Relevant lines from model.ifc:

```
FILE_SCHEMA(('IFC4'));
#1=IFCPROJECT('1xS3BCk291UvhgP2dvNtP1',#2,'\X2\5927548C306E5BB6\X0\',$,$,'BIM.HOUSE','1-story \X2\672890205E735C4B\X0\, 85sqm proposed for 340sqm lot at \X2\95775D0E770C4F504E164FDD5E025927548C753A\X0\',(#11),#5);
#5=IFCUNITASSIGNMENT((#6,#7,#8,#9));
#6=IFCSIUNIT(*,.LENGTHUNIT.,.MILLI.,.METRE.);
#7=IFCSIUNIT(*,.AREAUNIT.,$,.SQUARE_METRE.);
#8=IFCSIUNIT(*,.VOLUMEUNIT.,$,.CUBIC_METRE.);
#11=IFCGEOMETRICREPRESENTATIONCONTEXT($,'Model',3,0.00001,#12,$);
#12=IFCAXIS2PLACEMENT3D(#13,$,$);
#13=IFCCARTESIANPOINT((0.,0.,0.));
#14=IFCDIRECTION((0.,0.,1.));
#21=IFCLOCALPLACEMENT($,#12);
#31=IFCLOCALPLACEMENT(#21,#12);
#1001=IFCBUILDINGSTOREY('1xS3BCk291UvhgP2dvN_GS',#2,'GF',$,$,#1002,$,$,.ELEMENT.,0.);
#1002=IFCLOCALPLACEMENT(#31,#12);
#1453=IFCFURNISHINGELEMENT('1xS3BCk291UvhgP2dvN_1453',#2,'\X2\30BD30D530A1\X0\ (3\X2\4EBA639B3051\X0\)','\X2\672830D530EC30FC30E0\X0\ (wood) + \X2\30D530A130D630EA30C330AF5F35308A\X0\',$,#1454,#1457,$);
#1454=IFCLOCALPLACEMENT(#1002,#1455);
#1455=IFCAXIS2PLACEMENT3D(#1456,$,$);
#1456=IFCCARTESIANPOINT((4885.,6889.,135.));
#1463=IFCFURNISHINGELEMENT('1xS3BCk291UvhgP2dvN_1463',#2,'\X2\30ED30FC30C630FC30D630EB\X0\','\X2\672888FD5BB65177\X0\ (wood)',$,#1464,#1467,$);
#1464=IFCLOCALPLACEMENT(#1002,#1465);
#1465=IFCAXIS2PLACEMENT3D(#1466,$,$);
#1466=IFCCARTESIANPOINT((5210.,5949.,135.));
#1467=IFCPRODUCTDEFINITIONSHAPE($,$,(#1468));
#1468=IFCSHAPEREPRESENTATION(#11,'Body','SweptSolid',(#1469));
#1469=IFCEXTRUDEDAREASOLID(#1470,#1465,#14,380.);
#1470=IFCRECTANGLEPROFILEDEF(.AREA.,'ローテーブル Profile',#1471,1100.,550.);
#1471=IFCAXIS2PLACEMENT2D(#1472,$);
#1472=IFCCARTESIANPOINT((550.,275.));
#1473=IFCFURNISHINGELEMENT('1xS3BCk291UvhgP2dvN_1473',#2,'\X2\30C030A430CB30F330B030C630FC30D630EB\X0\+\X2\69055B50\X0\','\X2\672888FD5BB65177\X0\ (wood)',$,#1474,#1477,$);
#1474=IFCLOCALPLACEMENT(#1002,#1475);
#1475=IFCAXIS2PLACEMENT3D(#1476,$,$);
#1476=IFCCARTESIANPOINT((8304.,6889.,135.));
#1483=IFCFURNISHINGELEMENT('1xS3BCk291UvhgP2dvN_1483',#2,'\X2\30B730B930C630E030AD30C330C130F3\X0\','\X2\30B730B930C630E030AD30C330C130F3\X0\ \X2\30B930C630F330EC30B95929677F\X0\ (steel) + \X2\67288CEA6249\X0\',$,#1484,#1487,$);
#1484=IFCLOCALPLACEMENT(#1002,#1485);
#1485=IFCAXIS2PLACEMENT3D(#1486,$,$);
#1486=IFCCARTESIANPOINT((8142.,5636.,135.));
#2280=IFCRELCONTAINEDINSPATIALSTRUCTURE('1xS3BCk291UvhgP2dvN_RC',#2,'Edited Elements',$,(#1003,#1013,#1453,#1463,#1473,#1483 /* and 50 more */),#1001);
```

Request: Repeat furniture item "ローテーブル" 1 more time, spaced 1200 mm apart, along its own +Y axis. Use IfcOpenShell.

```python
import ifcopenshell
import ifcopenshell.api.geometry
import ifcopenshell.api.root
import ifcopenshell.util.element
import ifcopenshell.util.placement

model = ifcopenshell.open("model.ifc")


def reuse_history(source, copy):
    """copy_class also copies each property set's owner history, people and application; keep the originals."""
    for rel in copy.IsDefinedBy:
        if rel.is_a("IfcRelDefinesByProperties") and (history := rel.RelatingPropertyDefinition.OwnerHistory):
            rel.RelatingPropertyDefinition.OwnerHistory = source.OwnerHistory
            ifcopenshell.util.element.remove_deep2(model, history)


source = model.by_guid("1xS3BCk291UvhgP2dvN_1463")
base = ifcopenshell.util.placement.get_local_placement(source.ObjectPlacement)
step = base[:3, 1] * 1200.0

for i in range(1, 2):
    copy = ifcopenshell.api.root.copy_class(model, product=source)
    copy.Representation = ifcopenshell.util.element.copy_deep(
        model, source.Representation, exclude=["IfcGeometricRepresentationContext", "IfcRepresentationMap"]
    )
    reuse_history(source, copy)
    matrix = base.copy()
    matrix[:3, 3] += i * step
    print("added at", matrix[:3, 3].round(3) + 0.0)
    ifcopenshell.api.geometry.edit_object_placement(model, product=copy, matrix=matrix, is_si=False)

model.write("model_edited.ifc")
```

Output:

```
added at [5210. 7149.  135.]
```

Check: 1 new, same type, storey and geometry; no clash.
